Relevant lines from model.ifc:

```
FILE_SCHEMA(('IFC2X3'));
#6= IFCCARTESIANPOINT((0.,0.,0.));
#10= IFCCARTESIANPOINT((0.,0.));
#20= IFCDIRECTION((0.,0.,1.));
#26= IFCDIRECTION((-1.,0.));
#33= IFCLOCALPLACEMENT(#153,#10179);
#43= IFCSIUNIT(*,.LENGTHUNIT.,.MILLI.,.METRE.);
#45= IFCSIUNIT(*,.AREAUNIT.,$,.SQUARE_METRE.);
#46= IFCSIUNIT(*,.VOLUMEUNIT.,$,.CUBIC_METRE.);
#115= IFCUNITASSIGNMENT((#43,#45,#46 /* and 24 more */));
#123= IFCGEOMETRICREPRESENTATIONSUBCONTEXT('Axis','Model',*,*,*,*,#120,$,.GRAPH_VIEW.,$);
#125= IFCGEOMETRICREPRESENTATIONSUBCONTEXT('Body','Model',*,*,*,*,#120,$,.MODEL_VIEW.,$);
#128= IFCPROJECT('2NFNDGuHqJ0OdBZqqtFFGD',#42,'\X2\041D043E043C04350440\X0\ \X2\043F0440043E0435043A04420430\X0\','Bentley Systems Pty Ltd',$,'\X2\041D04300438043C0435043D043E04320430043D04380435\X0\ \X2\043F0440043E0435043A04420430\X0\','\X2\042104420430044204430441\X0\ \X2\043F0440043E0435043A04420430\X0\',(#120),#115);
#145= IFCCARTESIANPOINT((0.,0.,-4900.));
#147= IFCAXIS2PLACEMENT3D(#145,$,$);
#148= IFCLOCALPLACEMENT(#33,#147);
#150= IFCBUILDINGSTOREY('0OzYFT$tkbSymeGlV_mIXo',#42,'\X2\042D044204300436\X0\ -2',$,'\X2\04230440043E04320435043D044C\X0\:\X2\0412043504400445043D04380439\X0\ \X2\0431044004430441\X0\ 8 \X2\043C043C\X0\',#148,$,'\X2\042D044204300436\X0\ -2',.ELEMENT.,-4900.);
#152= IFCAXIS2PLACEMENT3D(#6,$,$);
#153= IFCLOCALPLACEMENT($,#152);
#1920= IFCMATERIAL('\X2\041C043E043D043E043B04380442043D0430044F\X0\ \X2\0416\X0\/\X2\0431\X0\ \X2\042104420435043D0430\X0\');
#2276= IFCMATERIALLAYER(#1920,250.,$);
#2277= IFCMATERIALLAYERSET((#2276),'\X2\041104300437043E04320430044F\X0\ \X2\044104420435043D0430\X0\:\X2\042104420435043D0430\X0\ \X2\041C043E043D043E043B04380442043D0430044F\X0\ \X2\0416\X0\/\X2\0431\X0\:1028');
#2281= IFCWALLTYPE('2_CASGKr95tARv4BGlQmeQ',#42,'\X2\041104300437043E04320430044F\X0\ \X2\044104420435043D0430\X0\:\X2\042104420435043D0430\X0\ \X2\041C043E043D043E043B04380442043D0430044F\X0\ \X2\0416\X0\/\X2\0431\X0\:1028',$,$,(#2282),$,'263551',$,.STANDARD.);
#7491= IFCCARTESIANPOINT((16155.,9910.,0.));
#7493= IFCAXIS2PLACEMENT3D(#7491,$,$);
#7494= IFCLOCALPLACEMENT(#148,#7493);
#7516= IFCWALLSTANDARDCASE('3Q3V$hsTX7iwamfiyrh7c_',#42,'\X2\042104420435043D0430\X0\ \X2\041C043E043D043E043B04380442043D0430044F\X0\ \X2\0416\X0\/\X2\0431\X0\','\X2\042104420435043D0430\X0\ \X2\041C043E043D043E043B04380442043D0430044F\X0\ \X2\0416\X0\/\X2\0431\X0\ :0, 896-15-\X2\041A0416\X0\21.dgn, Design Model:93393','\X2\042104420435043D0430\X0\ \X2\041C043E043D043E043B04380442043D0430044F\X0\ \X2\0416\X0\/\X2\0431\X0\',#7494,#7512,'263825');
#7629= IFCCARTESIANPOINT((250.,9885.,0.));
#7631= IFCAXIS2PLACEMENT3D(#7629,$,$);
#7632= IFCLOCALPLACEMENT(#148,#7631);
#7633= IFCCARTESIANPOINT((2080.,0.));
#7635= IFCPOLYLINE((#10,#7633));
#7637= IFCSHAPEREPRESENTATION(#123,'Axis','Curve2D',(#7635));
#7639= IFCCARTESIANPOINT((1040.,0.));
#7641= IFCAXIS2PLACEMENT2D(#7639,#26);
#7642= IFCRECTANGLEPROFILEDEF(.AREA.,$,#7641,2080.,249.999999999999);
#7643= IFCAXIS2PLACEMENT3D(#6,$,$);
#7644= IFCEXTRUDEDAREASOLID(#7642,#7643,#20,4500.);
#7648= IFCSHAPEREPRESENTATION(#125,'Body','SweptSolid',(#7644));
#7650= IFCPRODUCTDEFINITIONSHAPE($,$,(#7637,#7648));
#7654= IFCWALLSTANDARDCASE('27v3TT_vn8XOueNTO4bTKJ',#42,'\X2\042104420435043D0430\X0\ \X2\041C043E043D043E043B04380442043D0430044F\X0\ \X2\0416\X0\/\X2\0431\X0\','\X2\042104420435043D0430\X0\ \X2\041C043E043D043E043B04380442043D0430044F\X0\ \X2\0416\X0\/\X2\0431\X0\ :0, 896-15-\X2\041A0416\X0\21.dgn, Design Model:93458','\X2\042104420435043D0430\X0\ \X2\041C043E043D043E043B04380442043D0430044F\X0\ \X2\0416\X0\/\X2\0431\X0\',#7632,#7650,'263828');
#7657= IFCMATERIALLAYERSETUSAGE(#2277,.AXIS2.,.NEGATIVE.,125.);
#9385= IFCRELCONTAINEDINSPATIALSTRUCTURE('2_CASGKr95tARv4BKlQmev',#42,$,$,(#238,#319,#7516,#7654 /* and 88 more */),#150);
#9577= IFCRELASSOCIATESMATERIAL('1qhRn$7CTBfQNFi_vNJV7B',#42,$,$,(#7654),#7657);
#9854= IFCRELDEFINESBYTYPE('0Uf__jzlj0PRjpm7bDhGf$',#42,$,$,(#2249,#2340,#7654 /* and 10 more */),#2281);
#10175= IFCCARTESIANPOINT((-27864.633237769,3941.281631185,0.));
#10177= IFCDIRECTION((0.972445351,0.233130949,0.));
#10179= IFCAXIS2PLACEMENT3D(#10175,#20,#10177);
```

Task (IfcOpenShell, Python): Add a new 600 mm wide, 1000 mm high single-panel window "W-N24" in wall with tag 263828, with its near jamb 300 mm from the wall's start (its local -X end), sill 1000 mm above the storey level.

```python
import numpy as np
import ifcopenshell
import ifcopenshell.api.feature
import ifcopenshell.api.geometry
import ifcopenshell.api.root
import ifcopenshell.api.spatial
import ifcopenshell.api.type
import ifcopenshell.geom
import ifcopenshell.util.element
import ifcopenshell.util.placement
import ifcopenshell.util.representation
import ifcopenshell.util.shape
import ifcopenshell.util.unit

model = ifcopenshell.open("model.ifc")
unit_scale = ifcopenshell.util.unit.calculate_unit_scale(model)
settings = ifcopenshell.geom.settings()


def volume(element):
    """Net volume in cubic metres, openings subtracted."""
    shape = ifcopenshell.geom.create_shape(settings, element)
    return ifcopenshell.util.shape.get_volume(shape.geometry)


wall = model.by_guid("27v3TT_vn8XOueNTO4bTKJ")
storey = ifcopenshell.util.element.get_container(wall, ifc_class="IfcBuildingStorey")
context = ifcopenshell.util.representation.get_context(model, "Model", "Body", "MODEL_VIEW")
before = volume(wall)

width, height, from_end, sill = 0.6, 1, 0.3, 1  # metres

# The wall runs along its own X axis, and the end named is its -X end.
wall_shape = ifcopenshell.geom.create_shape(settings, wall)
x, y, z = ifcopenshell.util.shape.get_vertices(wall_shape.geometry).T
start = x.min() + from_end
face, thickness = float(y.min()), float(y.max() - y.min())
wall_matrix = ifcopenshell.util.placement.get_local_placement(wall.ObjectPlacement)
level = ifcopenshell.util.placement.get_local_placement(storey.ObjectPlacement)[2, 3]


def in_wall(x, y):
    """Placement at x, y metres in the wall's axes, at sill height."""
    matrix = wall_matrix.copy()
    matrix[:, 3] = wall_matrix @ np.array([x / unit_scale, y / unit_scale, 0.0, 1.0])
    matrix[2, 3] = level + sill / unit_scale
    return matrix


# Opening: a box that overshoots both wall faces by 50 mm.
opening = ifcopenshell.api.root.create_entity(model, ifc_class="IfcOpeningElement")
box = ifcopenshell.api.geometry.add_wall_representation(
    model, context=context, length=width, height=height, thickness=thickness + 0.1
)
ifcopenshell.api.geometry.assign_representation(model, product=opening, representation=box)
ifcopenshell.api.geometry.edit_object_placement(model, product=opening, matrix=in_wall(start, face - 0.05), is_si=False)
ifcopenshell.api.feature.add_feature(model, feature=opening, element=wall)

window = ifcopenshell.api.root.create_entity(model, ifc_class="IfcWindow", name="W-N24")
window.OverallWidth, window.OverallHeight = width / unit_scale, height / unit_scale
body = ifcopenshell.api.geometry.add_window_representation(
    model,
    context=context,
    overall_width=window.OverallWidth,
    overall_height=window.OverallHeight,
    partition_type="SINGLE_PANEL",
)
ifcopenshell.api.geometry.assign_representation(model, product=window, representation=body)
ifcopenshell.api.spatial.assign_container(model, products=[window], relating_structure=storey)
fills = ifcopenshell.api.feature.add_filling(model, opening=opening, element=window)
fills.OwnerHistory = window.OwnerHistory  # required in IFC2X3

# IFC2X3 keeps the operation on the window style.
style = ifcopenshell.api.root.create_entity(model, ifc_class="IfcWindowStyle", name="W-N24")
style.OperationType, style.ConstructionType = "SINGLE_PANEL", "NOTDEFINED"
style.ParameterTakesPrecedence = style.Sizeable = False
ifcopenshell.api.type.assign_type(model, related_objects=[window], relating_type=style)

# Centre the window in the wall's thickness.
ifcopenshell.api.geometry.edit_object_placement(model, product=window, matrix=in_wall(start, face), is_si=False)
window_shape = ifcopenshell.geom.create_shape(settings, window)
depth = ifcopenshell.util.shape.get_vertices(window_shape.geometry)[:, 1]
offset = face + thickness / 2 - (depth.min() + depth.max()) / 2
ifcopenshell.api.geometry.edit_object_placement(model, product=window, matrix=in_wall(start, offset), is_si=False)

after = volume(wall)

print(f"wall volume {before:.3f} -> {after:.3f} m3")

model.write("model-out.ifc")
```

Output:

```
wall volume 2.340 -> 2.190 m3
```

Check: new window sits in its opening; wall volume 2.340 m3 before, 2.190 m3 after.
